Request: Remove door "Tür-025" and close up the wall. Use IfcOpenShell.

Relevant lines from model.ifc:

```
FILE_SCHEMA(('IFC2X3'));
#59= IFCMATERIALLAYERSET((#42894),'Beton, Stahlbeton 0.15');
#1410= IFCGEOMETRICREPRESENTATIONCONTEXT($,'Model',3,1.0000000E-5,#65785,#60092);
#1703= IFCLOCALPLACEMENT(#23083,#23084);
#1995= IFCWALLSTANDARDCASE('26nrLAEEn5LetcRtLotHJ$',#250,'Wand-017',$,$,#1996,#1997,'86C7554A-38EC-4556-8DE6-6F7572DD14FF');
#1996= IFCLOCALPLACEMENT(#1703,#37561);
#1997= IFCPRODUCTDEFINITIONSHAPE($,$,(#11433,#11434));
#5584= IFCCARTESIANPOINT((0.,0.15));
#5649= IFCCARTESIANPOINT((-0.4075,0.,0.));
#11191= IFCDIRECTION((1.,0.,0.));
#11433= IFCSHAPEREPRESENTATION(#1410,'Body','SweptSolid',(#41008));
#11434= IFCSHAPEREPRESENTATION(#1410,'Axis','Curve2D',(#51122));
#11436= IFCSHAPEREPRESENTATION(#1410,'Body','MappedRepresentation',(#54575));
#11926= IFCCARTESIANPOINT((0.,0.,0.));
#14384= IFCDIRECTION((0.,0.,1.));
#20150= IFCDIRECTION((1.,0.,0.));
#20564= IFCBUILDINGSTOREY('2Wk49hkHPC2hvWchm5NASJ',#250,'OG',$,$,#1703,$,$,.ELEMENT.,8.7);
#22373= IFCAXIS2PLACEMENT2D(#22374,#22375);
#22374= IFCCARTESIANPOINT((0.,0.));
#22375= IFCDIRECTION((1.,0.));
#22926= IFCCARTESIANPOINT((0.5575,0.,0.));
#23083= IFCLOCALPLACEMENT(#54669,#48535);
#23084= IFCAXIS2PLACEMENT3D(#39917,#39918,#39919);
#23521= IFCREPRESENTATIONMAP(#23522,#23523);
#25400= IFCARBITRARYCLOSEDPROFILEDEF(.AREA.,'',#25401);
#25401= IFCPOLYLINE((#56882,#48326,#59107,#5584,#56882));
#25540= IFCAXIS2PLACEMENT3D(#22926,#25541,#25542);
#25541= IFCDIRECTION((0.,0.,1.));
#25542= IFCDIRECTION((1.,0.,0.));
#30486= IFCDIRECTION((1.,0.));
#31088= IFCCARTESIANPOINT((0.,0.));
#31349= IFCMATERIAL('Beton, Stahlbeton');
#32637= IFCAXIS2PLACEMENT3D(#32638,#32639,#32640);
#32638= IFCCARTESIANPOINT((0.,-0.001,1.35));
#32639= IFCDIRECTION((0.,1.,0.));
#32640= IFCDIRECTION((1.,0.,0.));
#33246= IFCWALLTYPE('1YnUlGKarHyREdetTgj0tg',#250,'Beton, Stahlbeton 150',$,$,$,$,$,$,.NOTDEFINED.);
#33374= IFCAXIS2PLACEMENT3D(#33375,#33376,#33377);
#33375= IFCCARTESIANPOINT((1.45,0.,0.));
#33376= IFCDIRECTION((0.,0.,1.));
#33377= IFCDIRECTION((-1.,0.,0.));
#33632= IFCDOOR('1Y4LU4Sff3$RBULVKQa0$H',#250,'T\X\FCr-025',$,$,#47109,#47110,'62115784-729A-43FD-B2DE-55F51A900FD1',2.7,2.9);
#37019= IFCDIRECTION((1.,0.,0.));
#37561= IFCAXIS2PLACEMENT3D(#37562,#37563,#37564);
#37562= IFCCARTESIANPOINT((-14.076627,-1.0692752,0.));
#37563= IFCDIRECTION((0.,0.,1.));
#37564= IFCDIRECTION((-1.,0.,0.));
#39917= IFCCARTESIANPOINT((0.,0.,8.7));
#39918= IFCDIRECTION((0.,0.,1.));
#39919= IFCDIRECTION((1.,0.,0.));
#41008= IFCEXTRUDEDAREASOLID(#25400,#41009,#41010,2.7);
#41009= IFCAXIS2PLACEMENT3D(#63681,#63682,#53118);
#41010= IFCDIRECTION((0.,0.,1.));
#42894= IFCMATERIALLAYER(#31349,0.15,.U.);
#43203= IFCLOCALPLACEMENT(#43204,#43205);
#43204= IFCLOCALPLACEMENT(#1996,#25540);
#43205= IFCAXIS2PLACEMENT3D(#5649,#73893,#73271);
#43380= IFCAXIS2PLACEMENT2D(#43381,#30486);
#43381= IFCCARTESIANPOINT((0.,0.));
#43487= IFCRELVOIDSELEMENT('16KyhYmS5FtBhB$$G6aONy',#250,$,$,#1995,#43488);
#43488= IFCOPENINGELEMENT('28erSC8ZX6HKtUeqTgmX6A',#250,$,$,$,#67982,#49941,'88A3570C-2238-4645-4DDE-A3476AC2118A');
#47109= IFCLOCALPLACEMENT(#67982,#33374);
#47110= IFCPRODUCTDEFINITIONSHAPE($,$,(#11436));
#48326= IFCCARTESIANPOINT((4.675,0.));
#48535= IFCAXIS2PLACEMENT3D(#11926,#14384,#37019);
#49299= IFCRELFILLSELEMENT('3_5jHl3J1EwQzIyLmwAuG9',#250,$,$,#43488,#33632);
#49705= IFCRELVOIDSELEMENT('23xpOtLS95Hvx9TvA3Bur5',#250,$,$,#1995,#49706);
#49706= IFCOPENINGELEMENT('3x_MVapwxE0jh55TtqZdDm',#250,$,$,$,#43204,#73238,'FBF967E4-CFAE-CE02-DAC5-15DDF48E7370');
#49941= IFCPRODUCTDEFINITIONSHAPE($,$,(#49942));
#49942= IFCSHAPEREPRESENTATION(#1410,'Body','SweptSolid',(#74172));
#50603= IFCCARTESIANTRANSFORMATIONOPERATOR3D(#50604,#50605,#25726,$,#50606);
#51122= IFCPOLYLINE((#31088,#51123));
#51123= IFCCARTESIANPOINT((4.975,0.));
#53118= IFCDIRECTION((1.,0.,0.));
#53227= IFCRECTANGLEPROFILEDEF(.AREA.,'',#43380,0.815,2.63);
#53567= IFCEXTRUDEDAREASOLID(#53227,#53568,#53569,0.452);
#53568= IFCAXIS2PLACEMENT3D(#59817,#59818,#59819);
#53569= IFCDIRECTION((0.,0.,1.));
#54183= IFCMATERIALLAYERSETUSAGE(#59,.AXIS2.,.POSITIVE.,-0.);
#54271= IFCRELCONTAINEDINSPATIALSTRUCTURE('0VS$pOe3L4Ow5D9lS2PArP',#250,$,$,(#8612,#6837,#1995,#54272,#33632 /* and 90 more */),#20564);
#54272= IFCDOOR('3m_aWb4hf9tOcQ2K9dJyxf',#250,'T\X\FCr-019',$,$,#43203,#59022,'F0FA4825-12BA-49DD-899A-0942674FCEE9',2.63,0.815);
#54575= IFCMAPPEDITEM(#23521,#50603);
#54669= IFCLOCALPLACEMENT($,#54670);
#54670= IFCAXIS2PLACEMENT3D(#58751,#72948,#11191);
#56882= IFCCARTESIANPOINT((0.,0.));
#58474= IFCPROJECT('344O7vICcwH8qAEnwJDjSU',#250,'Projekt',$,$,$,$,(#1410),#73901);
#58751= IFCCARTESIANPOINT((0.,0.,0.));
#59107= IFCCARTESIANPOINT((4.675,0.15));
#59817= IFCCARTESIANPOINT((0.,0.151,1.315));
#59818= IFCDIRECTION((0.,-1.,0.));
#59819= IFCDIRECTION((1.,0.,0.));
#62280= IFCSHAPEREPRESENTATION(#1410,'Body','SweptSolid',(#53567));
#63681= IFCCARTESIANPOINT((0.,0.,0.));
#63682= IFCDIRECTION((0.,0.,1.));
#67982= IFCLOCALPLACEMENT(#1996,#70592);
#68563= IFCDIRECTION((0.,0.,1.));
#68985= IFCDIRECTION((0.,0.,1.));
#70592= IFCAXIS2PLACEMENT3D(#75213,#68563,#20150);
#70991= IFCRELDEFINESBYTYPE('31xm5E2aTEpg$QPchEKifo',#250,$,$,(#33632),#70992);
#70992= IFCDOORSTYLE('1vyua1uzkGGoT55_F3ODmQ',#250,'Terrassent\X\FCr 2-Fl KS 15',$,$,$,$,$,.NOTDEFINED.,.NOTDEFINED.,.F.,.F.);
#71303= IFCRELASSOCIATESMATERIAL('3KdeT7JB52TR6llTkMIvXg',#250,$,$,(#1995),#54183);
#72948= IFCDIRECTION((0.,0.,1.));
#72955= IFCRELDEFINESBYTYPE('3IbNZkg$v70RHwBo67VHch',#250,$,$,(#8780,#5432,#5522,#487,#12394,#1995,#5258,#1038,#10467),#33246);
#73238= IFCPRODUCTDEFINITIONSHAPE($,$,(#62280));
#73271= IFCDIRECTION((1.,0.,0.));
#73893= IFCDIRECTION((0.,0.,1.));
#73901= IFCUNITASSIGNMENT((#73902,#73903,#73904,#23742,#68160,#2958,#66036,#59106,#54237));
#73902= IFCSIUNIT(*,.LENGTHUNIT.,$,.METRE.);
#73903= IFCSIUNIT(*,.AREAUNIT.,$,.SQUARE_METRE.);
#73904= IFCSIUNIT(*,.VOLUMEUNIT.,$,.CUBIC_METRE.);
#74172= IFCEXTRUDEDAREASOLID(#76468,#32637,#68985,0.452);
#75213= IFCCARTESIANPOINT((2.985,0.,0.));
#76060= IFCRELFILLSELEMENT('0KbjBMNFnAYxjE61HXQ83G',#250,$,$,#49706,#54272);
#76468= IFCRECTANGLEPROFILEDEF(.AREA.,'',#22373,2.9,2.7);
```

```python
import ifcopenshell
import ifcopenshell.api.feature
import ifcopenshell.api.root
import ifcopenshell.geom
import ifcopenshell.util.shape

model = ifcopenshell.open("model.ifc")
settings = ifcopenshell.geom.settings()


def volume(element):
    """Net volume in cubic metres, openings subtracted."""
    shape = ifcopenshell.geom.create_shape(settings, element)
    return ifcopenshell.util.shape.get_volume(shape.geometry)


door = model.by_guid("1Y4LU4Sff3$RBULVKQa0$H")
opening = door.FillsVoids[0].RelatingOpeningElement
wall = opening.VoidsElements[0].RelatingBuildingElement
before = volume(wall)

ifcopenshell.api.root.remove_product(model, product=door)
ifcopenshell.api.feature.remove_feature(model, feature=opening)

after = volume(wall)

print(f"wall volume {before:.3f} -> {after:.3f} m3")

model.write("model_updated.ifc")
```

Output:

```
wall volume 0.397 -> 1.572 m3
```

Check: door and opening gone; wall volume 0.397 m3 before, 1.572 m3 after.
